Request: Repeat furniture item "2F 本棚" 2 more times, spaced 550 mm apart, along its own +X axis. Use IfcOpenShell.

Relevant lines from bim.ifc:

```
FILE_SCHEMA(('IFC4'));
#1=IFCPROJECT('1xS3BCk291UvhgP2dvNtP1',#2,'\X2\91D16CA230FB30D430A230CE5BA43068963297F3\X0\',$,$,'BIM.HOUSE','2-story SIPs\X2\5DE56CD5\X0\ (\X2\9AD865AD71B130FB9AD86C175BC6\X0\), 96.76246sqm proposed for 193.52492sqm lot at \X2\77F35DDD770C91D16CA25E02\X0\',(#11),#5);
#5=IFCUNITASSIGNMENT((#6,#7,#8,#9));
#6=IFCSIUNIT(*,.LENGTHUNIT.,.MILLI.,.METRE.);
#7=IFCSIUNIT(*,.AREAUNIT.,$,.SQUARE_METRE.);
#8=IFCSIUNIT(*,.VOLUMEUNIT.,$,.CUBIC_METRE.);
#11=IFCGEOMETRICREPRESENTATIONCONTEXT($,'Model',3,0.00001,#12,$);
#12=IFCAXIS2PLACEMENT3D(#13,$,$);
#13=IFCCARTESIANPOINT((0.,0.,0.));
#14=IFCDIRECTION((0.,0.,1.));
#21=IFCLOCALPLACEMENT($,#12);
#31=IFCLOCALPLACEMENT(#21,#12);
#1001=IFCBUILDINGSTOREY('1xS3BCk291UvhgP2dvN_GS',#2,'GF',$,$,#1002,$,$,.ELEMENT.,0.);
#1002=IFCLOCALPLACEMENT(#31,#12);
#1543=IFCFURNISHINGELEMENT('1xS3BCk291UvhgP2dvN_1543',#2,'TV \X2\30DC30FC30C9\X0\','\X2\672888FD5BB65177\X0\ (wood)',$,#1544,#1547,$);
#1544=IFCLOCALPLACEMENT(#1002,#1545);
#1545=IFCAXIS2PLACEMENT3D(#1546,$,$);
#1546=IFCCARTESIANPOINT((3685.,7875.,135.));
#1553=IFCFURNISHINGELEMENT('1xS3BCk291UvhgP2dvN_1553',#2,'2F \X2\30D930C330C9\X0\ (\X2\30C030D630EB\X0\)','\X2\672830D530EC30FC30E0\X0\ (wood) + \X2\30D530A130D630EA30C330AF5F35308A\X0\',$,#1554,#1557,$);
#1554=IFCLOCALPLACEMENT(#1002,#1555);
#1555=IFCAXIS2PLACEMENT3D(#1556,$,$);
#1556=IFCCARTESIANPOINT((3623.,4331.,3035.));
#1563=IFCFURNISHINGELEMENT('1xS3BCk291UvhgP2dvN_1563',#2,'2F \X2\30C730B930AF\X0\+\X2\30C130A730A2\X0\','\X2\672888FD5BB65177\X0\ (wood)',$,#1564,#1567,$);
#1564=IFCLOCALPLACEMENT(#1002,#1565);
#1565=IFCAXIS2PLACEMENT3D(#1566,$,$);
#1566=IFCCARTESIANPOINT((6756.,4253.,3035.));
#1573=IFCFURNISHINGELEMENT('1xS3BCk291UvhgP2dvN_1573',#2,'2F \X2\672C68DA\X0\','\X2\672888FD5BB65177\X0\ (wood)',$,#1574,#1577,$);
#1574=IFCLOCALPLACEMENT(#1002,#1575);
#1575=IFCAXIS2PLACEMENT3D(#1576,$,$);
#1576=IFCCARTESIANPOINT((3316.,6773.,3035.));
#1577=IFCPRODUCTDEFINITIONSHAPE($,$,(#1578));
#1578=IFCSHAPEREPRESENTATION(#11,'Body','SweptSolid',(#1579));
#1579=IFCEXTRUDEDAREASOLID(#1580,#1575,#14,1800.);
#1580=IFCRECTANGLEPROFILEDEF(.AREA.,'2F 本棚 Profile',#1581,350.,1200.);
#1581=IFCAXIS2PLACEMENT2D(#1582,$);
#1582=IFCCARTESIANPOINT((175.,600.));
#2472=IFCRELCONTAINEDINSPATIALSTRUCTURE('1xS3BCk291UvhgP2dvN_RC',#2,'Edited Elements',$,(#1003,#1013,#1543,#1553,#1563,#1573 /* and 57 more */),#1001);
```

```python
import ifcopenshell
import ifcopenshell.api.geometry
import ifcopenshell.api.root
import ifcopenshell.util.element
import ifcopenshell.util.placement

model = ifcopenshell.open("bim.ifc")


def reuse_history(source, copy):
    """copy_class also copies each property set's owner history, people and application; keep the originals."""
    for rel in copy.IsDefinedBy:
        if rel.is_a("IfcRelDefinesByProperties") and (history := rel.RelatingPropertyDefinition.OwnerHistory):
            rel.RelatingPropertyDefinition.OwnerHistory = source.OwnerHistory
            ifcopenshell.util.element.remove_deep2(model, history)


source = model.by_guid("1xS3BCk291UvhgP2dvN_1573")
base = ifcopenshell.util.placement.get_local_placement(source.ObjectPlacement)
step = base[:3, 0] * 550.0

for i in range(1, 3):
    copy = ifcopenshell.api.root.copy_class(model, product=source)
    copy.Representation = ifcopenshell.util.element.copy_deep(
        model, source.Representation, exclude=["IfcGeometricRepresentationContext", "IfcRepresentationMap"]
    )
    reuse_history(source, copy)
    matrix = base.copy()
    matrix[:3, 3] += i * step
    print("added at", matrix[:3, 3].round(3) + 0.0)
    ifcopenshell.api.geometry.edit_object_placement(model, product=copy, matrix=matrix, is_si=False)

model.write("bim_rev.ifc")
```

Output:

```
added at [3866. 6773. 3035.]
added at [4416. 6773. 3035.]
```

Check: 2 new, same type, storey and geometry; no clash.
